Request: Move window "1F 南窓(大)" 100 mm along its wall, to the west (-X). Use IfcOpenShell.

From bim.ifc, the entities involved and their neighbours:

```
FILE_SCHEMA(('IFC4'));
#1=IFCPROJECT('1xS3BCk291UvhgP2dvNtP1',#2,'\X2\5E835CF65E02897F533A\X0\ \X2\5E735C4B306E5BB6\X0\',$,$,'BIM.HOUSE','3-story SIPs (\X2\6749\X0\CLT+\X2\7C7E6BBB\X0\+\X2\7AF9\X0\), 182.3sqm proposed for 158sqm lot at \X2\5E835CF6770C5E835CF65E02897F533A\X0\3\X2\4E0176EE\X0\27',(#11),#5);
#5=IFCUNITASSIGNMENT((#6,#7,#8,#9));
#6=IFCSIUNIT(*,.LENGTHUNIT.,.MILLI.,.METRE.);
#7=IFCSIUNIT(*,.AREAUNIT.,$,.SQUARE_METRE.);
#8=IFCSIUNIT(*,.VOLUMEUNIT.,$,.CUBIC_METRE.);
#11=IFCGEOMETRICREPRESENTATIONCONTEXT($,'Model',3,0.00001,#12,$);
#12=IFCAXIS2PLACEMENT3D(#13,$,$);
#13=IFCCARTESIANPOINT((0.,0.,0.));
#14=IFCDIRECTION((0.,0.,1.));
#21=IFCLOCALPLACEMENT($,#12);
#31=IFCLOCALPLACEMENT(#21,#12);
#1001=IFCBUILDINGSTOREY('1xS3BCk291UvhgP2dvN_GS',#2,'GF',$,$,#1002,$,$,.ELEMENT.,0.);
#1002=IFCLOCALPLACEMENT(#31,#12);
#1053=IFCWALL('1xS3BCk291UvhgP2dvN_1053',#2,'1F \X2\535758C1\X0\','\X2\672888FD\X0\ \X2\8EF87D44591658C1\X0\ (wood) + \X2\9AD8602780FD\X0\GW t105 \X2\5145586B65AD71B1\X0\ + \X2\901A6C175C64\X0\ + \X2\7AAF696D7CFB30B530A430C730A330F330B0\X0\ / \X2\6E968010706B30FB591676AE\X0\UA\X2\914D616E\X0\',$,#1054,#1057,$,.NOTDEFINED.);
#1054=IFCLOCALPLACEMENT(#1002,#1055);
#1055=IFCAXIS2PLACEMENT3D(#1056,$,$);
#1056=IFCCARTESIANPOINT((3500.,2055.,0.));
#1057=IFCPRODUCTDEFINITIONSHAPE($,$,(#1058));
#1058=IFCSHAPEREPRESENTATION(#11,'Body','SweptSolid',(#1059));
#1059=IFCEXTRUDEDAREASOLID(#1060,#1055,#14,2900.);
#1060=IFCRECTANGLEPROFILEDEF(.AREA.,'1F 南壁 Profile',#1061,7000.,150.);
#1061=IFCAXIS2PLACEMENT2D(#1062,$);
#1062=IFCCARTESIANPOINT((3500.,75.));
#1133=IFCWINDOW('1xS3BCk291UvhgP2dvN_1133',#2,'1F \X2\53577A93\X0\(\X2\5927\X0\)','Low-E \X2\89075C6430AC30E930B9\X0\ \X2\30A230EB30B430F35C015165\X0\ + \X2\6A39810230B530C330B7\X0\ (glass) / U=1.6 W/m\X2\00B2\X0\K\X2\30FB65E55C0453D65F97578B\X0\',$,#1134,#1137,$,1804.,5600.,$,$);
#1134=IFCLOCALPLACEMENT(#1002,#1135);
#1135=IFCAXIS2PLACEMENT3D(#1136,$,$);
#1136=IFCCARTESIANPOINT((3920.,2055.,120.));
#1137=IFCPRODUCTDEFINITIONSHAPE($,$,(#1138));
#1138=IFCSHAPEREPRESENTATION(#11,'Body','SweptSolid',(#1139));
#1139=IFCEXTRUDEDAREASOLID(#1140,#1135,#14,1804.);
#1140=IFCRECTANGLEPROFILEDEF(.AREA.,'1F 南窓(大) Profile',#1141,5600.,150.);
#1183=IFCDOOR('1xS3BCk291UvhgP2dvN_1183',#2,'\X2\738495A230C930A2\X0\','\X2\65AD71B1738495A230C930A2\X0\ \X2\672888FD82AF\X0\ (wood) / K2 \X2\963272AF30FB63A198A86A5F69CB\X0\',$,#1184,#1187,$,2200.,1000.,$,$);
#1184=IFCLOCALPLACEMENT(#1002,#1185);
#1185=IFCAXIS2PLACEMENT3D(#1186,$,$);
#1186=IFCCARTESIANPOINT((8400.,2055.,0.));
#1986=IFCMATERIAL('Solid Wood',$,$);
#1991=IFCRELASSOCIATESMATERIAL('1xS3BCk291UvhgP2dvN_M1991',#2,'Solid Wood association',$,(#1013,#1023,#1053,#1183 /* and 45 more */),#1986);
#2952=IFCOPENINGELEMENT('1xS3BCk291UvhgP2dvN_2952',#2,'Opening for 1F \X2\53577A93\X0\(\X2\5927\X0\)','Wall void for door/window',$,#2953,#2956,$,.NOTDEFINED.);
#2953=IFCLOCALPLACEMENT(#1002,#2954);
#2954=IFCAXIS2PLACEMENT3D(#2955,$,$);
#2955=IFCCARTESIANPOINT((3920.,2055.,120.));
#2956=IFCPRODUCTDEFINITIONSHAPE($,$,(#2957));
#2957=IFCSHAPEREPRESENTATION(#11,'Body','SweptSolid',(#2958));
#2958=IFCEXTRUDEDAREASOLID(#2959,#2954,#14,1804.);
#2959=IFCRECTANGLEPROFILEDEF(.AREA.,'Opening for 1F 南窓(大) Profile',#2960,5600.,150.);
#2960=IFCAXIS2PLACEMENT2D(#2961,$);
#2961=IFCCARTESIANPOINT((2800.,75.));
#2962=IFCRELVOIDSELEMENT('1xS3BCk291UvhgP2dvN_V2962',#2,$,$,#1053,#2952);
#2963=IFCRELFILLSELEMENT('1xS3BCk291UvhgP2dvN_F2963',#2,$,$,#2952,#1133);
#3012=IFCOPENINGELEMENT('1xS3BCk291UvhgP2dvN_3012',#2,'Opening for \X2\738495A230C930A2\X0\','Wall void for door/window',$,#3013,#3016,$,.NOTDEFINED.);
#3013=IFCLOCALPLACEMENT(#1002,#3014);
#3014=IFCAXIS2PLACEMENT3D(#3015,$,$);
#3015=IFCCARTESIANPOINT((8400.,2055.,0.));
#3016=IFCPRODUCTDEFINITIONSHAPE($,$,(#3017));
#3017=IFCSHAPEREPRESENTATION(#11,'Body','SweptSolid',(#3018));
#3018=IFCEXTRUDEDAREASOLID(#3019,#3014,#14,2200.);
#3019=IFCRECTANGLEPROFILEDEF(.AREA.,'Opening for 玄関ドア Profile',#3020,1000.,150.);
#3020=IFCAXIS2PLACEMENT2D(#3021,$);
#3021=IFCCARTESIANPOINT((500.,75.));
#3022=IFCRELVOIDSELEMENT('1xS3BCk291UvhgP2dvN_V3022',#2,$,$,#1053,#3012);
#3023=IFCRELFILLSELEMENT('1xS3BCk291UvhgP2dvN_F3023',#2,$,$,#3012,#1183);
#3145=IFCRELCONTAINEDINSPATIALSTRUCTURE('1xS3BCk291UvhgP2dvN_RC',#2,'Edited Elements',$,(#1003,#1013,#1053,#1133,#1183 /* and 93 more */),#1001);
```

```python
import ifcopenshell
import ifcopenshell.api.geometry
import ifcopenshell.util.placement
import ifcopenshell.util.unit

model = ifcopenshell.open("bim.ifc")
unit_scale = ifcopenshell.util.unit.calculate_unit_scale(model)

window = model.by_guid("1xS3BCk291UvhgP2dvN_1133")
opening = window.FillsVoids[0].RelatingOpeningElement
wall = opening.VoidsElements[0].RelatingBuildingElement

wall_matrix = ifcopenshell.util.placement.get_local_placement(wall.ObjectPlacement)
shift = wall_matrix[:3, 0] * -0.1 / unit_scale
before = ifcopenshell.util.placement.get_local_placement(window.ObjectPlacement)[:3, 3].copy()

# The window is not placed relative to its opening, so move both.
for product in (opening, window):
    matrix = ifcopenshell.util.placement.get_local_placement(product.ObjectPlacement)
    matrix[:3, 3] += shift
    ifcopenshell.api.geometry.edit_object_placement(model, product=product, matrix=matrix, is_si=False)

after = ifcopenshell.util.placement.get_local_placement(window.ObjectPlacement)[:3, 3]
print("window moved by", (after - before).round(3) + 0.0)

model.write("bim_rev.ifc")
```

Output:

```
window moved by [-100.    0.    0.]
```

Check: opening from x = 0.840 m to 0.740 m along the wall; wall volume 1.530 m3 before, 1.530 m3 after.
